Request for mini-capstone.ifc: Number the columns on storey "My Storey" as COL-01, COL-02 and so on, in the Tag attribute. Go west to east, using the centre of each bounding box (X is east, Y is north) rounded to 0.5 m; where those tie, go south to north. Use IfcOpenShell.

First a look at what the model holds.

```python
import ifcopenshell
import ifcopenshell.util.element
import ifcopenshell.util.placement

model = ifcopenshell.open("mini-capstone.ifc")
print(model.schema)
storey = next(s for s in model.by_type("IfcBuildingStorey") if s.Name == "My Storey")
columns = [e for e in ifcopenshell.util.element.get_decomposition(storey) if e.is_a("IfcColumn")]
for e in sorted(columns, key=lambda e: e.id()):
    origin = ifcopenshell.util.placement.get_local_placement(e.ObjectPlacement)[:3, 3]
    print(e.id(), e.Tag, e.Name, origin.round(2) + 0.0, sep=" | ")
```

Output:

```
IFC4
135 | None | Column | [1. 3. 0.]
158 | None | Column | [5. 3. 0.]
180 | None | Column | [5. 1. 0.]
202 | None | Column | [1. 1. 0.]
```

```python
import ifcopenshell
import ifcopenshell.geom
import ifcopenshell.util.element
import ifcopenshell.util.shape

model = ifcopenshell.open("mini-capstone.ifc")
settings = ifcopenshell.geom.settings()
settings.set("use-world-coords", True)


def centre(element):
    shape = ifcopenshell.geom.create_shape(settings, element)
    return ifcopenshell.util.shape.get_bbox_centroid(shape.geometry)


storey = next(s for s in model.by_type("IfcBuildingStorey") if s.Name == "My Storey")
columns = [e for e in ifcopenshell.util.element.get_decomposition(storey) if e.is_a("IfcColumn")]

# Insertion points can sit at a corner or the storey origin, so sort by the geometry (in metres).
centres = {e: centre(e) for e in columns}
columns.sort(key=lambda e: (round(centres[e][0] / 0.5), centres[e][1]))

for i, e in enumerate(columns, start=1):
    number = f"COL-{i:02d}"
    e.Tag = number
    print(e.id(), number)

model.write("mini-capstone_rev.ifc")
```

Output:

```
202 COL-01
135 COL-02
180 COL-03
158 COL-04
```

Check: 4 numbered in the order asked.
